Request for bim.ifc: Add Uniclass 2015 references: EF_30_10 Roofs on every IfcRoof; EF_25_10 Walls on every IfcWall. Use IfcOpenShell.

First a look at what the model holds.

```python
import ifcopenshell

model = ifcopenshell.open("bim.ifc")
print(model.schema)
print("classifications:", [c.Name for c in model.by_type("IfcClassification")])
for ifc_class in ("IfcDoor", "IfcRoof", "IfcStair", "IfcWall", "IfcWindow"):
    print(ifc_class, len(model.by_type(ifc_class)))
```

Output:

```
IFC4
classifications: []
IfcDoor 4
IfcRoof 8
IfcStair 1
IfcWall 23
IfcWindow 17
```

```python
import ifcopenshell
import ifcopenshell.api.classification

model = ifcopenshell.open("bim.ifc")

system = ifcopenshell.api.classification.add_classification(model, classification="Uniclass 2015")

codes = {
    "IfcRoof": ("EF_30_10", "Roofs"),
    "IfcWall": ("EF_25_10", "Walls"),
}
for ifc_class, (code, name) in codes.items():
    products = model.by_type(ifc_class)
    ifcopenshell.api.classification.add_reference(
        model, products=products, classification=system, identification=code, name=name
    )
    print(code, len(products))

model.write("bim_v2.ifc")
```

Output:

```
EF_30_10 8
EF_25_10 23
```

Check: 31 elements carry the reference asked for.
